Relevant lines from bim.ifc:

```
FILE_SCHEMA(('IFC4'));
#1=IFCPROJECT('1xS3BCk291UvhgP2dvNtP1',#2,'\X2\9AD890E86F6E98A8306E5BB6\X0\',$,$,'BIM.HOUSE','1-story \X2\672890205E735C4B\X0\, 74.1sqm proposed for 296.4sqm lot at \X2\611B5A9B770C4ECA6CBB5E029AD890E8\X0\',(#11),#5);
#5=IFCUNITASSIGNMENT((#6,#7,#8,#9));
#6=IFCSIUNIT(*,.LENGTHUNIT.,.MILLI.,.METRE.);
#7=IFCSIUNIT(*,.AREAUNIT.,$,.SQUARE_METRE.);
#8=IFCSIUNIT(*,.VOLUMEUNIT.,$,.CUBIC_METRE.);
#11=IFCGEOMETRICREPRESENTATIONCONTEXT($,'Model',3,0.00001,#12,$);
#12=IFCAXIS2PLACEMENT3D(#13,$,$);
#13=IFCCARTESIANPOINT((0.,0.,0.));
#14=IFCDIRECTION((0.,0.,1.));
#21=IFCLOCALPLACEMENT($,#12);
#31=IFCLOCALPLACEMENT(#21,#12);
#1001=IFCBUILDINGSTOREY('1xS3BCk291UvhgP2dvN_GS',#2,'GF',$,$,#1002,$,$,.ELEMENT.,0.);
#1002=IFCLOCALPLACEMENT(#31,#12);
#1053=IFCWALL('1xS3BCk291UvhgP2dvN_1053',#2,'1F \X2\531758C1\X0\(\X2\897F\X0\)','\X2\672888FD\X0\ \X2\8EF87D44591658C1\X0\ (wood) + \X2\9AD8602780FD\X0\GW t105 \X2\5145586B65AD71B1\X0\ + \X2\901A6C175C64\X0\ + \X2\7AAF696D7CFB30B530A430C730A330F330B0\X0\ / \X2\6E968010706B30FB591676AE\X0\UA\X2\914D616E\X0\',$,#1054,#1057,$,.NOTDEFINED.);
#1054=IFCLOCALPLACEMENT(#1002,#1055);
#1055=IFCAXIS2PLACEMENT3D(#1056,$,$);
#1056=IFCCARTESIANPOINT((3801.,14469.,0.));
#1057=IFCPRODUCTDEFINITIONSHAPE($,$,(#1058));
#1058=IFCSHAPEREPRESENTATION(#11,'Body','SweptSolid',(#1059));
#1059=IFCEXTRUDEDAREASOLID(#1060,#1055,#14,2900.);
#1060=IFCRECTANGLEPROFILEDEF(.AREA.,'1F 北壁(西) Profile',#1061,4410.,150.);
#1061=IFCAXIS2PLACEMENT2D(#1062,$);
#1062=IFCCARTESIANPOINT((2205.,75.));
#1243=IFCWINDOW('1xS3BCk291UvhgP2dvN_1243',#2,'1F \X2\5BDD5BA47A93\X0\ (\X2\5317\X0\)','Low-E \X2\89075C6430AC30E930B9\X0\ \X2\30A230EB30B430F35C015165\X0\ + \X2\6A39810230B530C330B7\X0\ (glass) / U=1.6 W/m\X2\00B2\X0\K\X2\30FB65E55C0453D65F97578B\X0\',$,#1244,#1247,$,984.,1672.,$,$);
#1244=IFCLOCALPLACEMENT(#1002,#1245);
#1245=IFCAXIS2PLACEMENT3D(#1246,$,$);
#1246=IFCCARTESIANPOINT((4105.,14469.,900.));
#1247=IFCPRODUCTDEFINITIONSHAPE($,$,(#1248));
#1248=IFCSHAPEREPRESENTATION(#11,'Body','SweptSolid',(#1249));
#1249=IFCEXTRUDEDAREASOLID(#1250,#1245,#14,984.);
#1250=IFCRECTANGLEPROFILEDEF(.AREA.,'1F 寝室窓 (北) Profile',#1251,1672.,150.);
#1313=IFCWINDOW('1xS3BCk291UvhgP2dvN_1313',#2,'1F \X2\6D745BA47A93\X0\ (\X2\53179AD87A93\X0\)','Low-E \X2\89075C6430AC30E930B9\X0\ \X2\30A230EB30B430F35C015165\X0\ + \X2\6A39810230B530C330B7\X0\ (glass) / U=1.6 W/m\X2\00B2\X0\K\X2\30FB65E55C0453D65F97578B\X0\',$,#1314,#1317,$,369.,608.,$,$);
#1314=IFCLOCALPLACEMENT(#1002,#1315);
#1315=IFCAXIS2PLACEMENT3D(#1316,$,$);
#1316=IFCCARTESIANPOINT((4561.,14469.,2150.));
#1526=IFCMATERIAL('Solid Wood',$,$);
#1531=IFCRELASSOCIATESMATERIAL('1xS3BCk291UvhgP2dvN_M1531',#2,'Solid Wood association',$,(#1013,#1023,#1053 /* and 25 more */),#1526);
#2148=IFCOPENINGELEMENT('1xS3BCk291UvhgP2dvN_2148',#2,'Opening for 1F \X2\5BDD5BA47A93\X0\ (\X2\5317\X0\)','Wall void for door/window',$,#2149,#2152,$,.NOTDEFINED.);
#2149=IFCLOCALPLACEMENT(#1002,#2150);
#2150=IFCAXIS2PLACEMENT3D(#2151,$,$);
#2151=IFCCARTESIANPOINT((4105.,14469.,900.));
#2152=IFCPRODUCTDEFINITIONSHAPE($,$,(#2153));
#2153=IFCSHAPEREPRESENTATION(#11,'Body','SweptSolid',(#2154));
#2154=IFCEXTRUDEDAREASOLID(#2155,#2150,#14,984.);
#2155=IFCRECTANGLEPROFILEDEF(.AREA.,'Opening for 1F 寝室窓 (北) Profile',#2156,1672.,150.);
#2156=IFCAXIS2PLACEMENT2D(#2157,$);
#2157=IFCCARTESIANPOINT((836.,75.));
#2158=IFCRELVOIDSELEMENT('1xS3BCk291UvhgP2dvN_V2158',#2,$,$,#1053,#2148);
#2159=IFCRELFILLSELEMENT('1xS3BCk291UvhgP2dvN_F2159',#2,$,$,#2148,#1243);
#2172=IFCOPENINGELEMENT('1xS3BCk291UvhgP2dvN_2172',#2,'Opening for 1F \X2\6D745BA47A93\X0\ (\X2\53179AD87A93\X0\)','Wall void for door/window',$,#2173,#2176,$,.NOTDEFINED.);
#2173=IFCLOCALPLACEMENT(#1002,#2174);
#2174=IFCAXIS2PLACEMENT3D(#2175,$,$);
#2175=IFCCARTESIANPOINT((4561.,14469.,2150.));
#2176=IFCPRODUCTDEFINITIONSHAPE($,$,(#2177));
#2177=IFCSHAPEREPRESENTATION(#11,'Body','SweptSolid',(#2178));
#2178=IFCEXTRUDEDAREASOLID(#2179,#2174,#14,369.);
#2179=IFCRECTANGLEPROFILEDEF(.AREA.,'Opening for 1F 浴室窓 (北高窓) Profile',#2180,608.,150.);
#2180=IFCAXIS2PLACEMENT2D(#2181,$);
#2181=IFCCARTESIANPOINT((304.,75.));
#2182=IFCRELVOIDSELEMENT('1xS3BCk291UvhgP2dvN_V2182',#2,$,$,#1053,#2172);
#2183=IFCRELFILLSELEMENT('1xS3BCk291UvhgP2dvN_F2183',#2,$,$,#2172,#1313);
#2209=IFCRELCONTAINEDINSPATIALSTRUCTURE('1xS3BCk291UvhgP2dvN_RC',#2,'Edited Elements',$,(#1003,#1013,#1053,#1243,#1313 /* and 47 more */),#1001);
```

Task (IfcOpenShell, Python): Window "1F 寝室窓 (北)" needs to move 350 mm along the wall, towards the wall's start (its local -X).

```python
import ifcopenshell
import ifcopenshell.api.geometry
import ifcopenshell.util.placement

model = ifcopenshell.open("bim.ifc")

window = model.by_guid("1xS3BCk291UvhgP2dvN_1243")
opening = window.FillsVoids[0].RelatingOpeningElement
wall = opening.VoidsElements[0].RelatingBuildingElement

wall_matrix = ifcopenshell.util.placement.get_local_placement(wall.ObjectPlacement)
shift = wall_matrix[:3, 0] * -350.0
before = ifcopenshell.util.placement.get_local_placement(window.ObjectPlacement)[:3, 3].copy()

# The window is not placed relative to its opening, so move both.
for product in (opening, window):
    matrix = ifcopenshell.util.placement.get_local_placement(product.ObjectPlacement)
    matrix[:3, 3] += shift
    ifcopenshell.api.geometry.edit_object_placement(model, product=product, matrix=matrix, is_si=False)

after = ifcopenshell.util.placement.get_local_placement(window.ObjectPlacement)[:3, 3]
print("window moved by", (after - before).round(3) + 0.0)

model.write("bim_edited.ifc")
```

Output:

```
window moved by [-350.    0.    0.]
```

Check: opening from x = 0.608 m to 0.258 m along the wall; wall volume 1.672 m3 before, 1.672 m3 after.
